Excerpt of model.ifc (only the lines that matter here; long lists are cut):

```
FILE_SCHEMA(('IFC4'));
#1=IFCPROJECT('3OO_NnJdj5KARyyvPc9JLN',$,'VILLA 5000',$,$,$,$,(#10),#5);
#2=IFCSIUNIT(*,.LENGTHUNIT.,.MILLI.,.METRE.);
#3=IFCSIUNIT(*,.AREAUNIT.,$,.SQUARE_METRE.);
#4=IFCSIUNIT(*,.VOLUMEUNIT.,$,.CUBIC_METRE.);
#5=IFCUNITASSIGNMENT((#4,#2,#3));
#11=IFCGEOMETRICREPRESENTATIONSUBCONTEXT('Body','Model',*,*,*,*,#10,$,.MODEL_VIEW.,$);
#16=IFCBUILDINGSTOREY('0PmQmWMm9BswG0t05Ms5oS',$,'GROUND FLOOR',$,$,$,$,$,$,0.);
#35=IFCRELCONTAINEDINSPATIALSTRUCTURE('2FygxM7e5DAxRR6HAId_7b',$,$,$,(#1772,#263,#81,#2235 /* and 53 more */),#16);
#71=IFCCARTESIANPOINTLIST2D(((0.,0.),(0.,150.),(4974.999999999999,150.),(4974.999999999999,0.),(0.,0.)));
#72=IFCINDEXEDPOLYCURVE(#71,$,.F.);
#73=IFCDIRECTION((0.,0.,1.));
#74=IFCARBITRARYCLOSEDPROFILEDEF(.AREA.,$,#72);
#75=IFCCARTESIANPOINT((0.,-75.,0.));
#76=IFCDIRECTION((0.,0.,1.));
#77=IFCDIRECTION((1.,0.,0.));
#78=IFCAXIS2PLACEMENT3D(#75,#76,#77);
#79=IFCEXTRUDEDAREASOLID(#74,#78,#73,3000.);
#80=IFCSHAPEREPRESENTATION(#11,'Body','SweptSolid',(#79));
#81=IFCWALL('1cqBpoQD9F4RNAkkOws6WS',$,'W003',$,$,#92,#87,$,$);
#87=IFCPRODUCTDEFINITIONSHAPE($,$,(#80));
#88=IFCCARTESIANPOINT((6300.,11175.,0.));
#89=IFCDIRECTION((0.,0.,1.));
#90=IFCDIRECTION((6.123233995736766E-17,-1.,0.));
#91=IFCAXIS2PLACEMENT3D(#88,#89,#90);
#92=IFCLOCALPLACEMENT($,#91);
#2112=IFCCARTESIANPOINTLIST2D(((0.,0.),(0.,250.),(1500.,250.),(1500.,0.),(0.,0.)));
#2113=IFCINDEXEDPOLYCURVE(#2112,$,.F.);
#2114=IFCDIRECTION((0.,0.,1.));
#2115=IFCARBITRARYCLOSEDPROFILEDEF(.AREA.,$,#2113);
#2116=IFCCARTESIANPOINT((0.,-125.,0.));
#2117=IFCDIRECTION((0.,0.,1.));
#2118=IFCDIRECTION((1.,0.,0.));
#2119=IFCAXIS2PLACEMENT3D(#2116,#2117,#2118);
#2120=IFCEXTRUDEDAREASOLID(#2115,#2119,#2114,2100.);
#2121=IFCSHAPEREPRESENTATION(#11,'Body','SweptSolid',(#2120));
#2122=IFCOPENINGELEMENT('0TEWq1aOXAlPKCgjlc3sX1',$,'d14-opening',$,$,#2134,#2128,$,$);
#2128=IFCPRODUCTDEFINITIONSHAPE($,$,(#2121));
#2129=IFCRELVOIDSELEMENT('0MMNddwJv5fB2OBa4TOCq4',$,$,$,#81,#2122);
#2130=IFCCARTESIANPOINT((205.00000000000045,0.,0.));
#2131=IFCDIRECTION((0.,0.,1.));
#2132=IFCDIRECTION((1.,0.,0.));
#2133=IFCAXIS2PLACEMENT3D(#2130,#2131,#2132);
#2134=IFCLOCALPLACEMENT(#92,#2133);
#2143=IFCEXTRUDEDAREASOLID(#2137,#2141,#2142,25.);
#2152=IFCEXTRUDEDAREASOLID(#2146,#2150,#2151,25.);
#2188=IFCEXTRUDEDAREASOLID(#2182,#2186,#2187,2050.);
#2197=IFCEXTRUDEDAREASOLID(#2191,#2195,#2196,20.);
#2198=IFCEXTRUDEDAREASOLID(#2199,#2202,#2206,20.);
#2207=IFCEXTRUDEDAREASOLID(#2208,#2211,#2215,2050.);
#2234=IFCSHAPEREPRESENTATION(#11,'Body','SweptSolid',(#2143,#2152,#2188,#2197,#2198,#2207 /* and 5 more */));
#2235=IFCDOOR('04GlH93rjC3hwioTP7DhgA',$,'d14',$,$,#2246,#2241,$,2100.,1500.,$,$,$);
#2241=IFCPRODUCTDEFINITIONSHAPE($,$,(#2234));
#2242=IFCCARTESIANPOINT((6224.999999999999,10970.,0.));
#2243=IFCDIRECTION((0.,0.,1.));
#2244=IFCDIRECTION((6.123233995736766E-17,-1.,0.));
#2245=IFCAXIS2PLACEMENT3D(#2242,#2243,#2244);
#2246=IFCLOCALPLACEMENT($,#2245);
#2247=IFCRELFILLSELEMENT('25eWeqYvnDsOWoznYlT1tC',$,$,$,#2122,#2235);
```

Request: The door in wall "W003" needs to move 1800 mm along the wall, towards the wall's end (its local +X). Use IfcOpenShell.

```python
import ifcopenshell
import ifcopenshell.api.geometry
import ifcopenshell.util.placement
import ifcopenshell.util.unit

model = ifcopenshell.open("model.ifc")
unit_scale = ifcopenshell.util.unit.calculate_unit_scale(model)

door = model.by_guid("04GlH93rjC3hwioTP7DhgA")
opening = door.FillsVoids[0].RelatingOpeningElement
wall = opening.VoidsElements[0].RelatingBuildingElement

wall_matrix = ifcopenshell.util.placement.get_local_placement(wall.ObjectPlacement)
shift = wall_matrix[:3, 0] * 1.8 / unit_scale
before = ifcopenshell.util.placement.get_local_placement(door.ObjectPlacement)[:3, 3].copy()

# The door is not placed relative to its opening, so move both.
for product in (opening, door):
    matrix = ifcopenshell.util.placement.get_local_placement(product.ObjectPlacement)
    matrix[:3, 3] += shift
    ifcopenshell.api.geometry.edit_object_placement(model, product=product, matrix=matrix, is_si=False)

after = ifcopenshell.util.placement.get_local_placement(door.ObjectPlacement)[:3, 3]
print("door moved by", (after - before).round(3) + 0.0)

model.write("model_updated.ifc")
```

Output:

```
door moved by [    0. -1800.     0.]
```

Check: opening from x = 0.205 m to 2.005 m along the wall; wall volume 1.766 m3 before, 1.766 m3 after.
